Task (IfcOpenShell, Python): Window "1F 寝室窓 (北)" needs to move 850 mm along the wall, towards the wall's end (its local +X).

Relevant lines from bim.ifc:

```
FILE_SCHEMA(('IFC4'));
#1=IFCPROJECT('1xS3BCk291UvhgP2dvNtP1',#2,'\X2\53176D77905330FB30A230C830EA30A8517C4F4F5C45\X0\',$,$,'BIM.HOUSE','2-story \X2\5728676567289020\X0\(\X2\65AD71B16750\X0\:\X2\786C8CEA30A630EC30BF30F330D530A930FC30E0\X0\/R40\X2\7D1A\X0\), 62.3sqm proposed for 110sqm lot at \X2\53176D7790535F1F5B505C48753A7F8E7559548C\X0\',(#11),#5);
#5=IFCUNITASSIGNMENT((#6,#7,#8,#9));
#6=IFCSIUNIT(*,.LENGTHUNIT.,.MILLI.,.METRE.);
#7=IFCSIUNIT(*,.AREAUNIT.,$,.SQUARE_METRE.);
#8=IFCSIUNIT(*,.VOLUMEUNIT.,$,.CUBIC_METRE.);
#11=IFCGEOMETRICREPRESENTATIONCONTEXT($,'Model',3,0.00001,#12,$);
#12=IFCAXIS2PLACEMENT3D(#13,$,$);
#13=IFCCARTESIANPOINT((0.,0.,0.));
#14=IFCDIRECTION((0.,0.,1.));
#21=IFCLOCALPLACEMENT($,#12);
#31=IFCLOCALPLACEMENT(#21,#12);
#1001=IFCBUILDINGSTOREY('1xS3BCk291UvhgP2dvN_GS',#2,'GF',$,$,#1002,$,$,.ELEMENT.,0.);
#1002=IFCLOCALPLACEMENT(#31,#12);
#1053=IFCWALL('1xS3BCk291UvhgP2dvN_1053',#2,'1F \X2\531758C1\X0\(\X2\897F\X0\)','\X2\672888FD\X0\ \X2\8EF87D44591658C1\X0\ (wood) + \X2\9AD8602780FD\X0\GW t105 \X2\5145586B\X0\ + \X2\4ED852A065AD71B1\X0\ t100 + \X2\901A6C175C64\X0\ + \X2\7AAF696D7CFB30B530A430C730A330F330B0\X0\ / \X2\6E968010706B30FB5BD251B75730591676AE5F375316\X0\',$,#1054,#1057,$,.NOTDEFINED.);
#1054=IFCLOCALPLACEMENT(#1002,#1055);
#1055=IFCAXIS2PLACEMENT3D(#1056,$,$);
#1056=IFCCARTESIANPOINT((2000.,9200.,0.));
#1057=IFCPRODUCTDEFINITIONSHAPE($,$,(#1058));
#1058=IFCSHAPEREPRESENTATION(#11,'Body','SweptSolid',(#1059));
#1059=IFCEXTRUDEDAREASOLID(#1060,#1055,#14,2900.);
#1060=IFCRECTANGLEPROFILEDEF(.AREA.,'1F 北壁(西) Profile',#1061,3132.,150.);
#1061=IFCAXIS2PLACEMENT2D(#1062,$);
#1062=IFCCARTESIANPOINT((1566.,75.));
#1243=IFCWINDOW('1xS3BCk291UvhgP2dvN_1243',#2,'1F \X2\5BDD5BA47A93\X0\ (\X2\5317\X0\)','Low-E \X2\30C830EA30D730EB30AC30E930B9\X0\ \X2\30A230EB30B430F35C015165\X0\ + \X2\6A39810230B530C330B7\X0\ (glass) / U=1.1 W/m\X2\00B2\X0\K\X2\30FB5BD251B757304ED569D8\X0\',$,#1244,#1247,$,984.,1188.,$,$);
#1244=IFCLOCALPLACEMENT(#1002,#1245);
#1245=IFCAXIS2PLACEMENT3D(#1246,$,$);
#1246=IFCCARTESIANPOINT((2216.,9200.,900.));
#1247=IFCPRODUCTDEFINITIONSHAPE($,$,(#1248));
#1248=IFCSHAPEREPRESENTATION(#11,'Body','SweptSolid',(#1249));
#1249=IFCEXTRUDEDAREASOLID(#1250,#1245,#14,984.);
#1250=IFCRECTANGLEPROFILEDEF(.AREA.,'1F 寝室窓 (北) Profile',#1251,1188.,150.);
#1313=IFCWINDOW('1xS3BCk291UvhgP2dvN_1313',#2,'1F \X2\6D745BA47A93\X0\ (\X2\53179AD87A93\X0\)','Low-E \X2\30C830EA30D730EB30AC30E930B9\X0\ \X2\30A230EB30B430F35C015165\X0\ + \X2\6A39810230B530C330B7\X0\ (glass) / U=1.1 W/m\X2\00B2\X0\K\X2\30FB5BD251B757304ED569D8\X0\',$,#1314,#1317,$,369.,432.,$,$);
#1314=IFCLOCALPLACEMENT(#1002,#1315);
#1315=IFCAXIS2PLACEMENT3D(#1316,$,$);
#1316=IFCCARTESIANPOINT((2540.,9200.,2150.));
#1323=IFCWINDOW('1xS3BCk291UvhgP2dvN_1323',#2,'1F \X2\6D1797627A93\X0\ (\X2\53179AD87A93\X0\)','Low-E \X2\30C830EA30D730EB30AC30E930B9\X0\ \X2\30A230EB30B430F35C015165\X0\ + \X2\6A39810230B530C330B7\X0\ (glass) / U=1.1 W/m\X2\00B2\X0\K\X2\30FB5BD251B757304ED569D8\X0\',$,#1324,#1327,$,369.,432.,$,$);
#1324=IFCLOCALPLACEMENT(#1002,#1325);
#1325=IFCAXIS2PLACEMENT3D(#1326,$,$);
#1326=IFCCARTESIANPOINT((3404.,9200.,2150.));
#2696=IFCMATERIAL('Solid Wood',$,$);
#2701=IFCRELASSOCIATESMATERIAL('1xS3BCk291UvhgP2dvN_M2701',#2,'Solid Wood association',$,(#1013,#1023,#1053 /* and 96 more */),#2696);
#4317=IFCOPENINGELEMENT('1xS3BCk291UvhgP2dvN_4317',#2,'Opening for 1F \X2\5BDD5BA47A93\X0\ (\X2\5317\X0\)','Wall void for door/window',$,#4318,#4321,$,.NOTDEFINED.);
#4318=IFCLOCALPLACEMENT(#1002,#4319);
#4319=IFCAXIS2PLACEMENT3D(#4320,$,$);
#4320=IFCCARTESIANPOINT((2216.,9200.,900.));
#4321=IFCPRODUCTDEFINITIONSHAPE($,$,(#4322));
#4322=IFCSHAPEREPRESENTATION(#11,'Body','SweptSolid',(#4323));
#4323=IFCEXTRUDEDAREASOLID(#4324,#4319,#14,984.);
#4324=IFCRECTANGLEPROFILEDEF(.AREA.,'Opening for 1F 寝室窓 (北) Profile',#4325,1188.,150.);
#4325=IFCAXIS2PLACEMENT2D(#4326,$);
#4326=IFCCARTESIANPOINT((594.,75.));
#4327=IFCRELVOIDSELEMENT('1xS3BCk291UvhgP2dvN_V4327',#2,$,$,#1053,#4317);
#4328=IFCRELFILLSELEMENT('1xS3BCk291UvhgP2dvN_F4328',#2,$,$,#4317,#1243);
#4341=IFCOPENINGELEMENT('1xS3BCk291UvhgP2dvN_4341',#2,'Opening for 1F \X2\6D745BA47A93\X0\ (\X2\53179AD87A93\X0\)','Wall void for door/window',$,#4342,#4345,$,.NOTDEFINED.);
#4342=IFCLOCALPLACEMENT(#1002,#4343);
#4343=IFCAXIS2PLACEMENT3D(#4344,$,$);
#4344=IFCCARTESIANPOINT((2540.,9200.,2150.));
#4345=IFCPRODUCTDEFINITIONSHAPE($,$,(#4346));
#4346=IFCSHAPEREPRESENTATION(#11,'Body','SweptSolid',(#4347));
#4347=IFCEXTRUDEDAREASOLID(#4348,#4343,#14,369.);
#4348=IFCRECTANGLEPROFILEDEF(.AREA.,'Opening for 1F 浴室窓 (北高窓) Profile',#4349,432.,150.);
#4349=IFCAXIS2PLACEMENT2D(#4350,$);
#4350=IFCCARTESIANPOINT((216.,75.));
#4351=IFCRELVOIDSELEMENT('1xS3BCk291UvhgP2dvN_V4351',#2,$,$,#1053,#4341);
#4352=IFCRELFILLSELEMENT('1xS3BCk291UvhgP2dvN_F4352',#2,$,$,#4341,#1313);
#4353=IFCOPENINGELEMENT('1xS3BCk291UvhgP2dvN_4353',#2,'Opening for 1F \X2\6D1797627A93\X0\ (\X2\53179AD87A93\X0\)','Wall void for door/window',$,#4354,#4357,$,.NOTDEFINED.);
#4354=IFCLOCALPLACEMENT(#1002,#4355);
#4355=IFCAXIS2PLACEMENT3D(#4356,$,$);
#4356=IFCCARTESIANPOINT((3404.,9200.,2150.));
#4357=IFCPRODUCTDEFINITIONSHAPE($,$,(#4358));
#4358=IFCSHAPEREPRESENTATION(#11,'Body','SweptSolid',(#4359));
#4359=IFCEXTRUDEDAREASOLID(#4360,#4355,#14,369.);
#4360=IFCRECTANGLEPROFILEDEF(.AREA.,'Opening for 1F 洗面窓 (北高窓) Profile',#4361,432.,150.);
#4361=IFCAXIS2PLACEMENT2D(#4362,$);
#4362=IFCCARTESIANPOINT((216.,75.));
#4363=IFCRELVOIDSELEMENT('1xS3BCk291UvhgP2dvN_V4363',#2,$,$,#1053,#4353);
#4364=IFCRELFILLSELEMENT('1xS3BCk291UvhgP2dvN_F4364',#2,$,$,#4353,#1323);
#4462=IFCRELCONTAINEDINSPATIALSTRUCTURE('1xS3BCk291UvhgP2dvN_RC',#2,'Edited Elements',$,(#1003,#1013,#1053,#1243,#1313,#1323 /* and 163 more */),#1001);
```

```python
import ifcopenshell
import ifcopenshell.api.geometry
import ifcopenshell.util.placement
import ifcopenshell.util.unit

model = ifcopenshell.open("bim.ifc")
unit_scale = ifcopenshell.util.unit.calculate_unit_scale(model)

window = model.by_id(1243)
opening = window.FillsVoids[0].RelatingOpeningElement
wall = opening.VoidsElements[0].RelatingBuildingElement

wall_matrix = ifcopenshell.util.placement.get_local_placement(wall.ObjectPlacement)
shift = wall_matrix[:3, 0] * 0.85 / unit_scale
before = ifcopenshell.util.placement.get_local_placement(window.ObjectPlacement)[:3, 3].copy()

# The window is not placed relative to its opening, so move both.
for product in (opening, window):
    matrix = ifcopenshell.util.placement.get_local_placement(product.ObjectPlacement)
    matrix[:3, 3] += shift
    ifcopenshell.api.geometry.edit_object_placement(model, product=product, matrix=matrix, is_si=False)

after = ifcopenshell.util.placement.get_local_placement(window.ObjectPlacement)[:3, 3]
print("window moved by", (after - before).round(3) + 0.0)

model.write("bim-out.ifc")
```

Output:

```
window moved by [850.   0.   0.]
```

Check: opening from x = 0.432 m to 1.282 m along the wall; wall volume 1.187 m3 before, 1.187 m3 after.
